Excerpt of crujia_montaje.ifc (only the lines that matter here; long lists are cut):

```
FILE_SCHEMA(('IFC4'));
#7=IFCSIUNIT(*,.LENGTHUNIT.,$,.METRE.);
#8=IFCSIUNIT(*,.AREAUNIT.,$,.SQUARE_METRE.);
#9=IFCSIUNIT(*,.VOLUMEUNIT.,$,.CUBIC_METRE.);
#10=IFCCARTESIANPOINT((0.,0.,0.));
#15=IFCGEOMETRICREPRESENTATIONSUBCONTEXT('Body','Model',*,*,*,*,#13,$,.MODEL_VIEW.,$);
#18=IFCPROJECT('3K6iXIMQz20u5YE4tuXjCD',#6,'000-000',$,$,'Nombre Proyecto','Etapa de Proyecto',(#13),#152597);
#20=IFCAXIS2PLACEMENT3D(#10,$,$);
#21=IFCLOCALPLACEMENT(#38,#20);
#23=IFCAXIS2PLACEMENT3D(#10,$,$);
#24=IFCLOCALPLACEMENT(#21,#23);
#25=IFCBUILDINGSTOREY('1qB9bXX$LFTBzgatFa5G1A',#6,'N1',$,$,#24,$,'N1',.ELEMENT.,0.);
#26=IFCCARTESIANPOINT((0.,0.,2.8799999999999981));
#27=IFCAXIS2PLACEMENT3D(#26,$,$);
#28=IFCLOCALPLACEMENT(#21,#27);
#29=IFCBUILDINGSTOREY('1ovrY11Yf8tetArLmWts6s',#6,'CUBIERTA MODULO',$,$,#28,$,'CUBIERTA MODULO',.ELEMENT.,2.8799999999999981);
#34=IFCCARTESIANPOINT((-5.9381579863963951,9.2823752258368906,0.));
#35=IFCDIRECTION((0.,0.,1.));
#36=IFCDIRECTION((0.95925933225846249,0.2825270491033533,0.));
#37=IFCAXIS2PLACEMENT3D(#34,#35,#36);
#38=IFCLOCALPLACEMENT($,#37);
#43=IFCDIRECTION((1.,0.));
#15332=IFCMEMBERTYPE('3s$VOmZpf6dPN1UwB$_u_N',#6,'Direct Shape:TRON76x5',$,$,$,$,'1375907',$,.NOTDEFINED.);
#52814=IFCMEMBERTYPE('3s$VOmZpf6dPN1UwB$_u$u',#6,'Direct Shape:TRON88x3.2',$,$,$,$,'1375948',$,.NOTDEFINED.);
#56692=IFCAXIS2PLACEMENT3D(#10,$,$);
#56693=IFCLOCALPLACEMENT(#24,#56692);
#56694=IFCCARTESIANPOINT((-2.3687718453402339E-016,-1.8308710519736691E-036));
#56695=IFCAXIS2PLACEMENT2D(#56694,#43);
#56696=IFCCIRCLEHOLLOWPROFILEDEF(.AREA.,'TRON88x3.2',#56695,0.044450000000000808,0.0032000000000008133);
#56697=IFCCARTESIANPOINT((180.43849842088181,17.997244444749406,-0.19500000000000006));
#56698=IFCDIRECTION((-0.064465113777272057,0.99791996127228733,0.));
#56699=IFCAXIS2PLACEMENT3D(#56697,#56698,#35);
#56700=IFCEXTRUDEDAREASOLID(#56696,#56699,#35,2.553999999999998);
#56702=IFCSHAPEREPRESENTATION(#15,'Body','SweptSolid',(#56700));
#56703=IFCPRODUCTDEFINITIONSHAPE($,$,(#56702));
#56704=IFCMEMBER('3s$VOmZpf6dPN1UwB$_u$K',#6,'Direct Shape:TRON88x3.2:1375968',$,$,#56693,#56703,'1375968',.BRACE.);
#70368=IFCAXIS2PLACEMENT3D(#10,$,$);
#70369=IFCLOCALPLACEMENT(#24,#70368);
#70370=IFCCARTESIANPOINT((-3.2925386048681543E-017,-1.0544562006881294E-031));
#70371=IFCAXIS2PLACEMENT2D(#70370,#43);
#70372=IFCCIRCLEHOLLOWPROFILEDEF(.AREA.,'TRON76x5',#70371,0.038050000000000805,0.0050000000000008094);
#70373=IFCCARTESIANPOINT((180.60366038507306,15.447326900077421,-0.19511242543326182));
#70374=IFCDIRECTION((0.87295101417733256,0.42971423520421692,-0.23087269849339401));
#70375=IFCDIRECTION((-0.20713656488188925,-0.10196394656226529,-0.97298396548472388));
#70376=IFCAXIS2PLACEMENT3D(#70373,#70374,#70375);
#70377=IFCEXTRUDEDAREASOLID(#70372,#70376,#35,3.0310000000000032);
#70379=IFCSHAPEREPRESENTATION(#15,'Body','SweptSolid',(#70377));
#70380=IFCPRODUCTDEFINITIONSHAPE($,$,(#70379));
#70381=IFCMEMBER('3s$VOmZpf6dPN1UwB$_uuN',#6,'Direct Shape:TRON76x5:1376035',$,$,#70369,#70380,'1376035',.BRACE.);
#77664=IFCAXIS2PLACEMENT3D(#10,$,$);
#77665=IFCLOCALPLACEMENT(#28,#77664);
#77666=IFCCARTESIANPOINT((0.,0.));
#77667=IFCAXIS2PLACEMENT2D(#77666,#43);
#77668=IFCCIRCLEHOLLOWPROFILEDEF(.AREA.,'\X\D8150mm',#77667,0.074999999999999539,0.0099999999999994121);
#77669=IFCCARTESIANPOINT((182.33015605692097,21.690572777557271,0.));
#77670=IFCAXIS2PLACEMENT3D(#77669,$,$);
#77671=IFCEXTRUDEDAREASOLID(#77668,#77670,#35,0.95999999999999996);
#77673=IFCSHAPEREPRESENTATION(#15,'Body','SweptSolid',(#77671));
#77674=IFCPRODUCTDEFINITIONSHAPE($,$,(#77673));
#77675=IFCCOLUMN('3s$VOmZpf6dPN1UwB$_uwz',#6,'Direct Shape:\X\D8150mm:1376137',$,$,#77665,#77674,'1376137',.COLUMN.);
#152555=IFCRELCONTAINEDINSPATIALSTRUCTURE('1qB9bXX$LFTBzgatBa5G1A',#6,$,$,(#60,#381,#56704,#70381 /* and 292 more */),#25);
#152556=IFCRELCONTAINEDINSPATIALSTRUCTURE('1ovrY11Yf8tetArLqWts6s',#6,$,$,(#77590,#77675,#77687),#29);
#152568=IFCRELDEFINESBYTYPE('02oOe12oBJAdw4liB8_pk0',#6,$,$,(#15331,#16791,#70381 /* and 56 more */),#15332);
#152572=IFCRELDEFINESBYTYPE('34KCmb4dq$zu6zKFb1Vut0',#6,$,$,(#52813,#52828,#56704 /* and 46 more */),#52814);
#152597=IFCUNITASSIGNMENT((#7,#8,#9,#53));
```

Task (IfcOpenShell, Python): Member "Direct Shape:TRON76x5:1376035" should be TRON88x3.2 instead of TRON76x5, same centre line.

```python
import ifcopenshell
import ifcopenshell.api.type
import ifcopenshell.util.element
import ifcopenshell.util.representation

model = ifcopenshell.open("crujia_montaje.ifc")

member = model.by_guid("3s$VOmZpf6dPN1UwB$_uuN")
source = next(p for p in model.by_type("IfcCircleHollowProfileDef") if p.ProfileName == "TRON88x3.2")

body = ifcopenshell.util.representation.get_representation(member, "Model", "Body")
solid = body.Items[0]
old_profile = solid.SweptArea

# Copy the section's sizes but keep this member's own profile position.
profile = ifcopenshell.util.element.copy(model, source)
profile.Position = old_profile.Position
solid.SweptArea = profile
if not model.get_total_inverses(old_profile):
    ifcopenshell.util.element.remove_deep2(model, old_profile)

new_type = model.by_guid("3s$VOmZpf6dPN1UwB$_u$u")
ifcopenshell.api.type.assign_type(
    model, related_objects=[member], relating_type=new_type, should_map_representations=False
)
member.Name = member.Name.replace("TRON76x5", "TRON88x3.2")

print(solid.SweptArea)

model.write("crujia_montaje_v2.ifc")
```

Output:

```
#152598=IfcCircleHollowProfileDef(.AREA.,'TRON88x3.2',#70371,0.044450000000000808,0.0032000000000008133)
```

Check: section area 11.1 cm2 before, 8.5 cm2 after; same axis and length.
